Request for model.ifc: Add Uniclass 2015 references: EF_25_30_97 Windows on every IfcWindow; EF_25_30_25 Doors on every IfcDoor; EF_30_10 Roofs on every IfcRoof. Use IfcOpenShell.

First a look at what the model holds.

```python
import ifcopenshell

model = ifcopenshell.open("model.ifc")
print(model.schema)
print("classifications:", [c.Name for c in model.by_type("IfcClassification")])
for ifc_class in ("IfcDoor", "IfcRoof", "IfcStair", "IfcWall", "IfcWindow"):
    print(ifc_class, len(model.by_type(ifc_class)))
```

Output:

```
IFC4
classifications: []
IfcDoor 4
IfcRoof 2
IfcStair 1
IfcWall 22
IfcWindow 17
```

```python
import ifcopenshell
import ifcopenshell.api.classification

model = ifcopenshell.open("model.ifc")

system = ifcopenshell.api.classification.add_classification(model, classification="Uniclass 2015")

codes = {
    "IfcWindow": ("EF_25_30_97", "Windows"),
    "IfcDoor": ("EF_25_30_25", "Doors"),
    "IfcRoof": ("EF_30_10", "Roofs"),
}
for ifc_class, (code, name) in codes.items():
    products = model.by_type(ifc_class)
    ifcopenshell.api.classification.add_reference(
        model, products=products, classification=system, identification=code, name=name
    )
    print(code, len(products))

model.write("model_v2.ifc")
```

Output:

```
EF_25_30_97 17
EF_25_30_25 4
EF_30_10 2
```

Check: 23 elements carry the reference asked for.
